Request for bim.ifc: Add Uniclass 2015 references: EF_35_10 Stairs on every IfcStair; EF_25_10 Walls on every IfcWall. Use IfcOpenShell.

First a look at what the model holds.

```python
import ifcopenshell

model = ifcopenshell.open("bim.ifc")
print(model.schema)
print("classifications:", [c.Name for c in model.by_type("IfcClassification")])
for ifc_class in ("IfcDoor", "IfcRoof", "IfcStair", "IfcWall", "IfcWindow"):
    print(ifc_class, len(model.by_type(ifc_class)))
```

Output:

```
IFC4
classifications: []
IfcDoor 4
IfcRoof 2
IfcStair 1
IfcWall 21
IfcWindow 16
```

```python
import ifcopenshell
import ifcopenshell.api.classification

model = ifcopenshell.open("bim.ifc")

system = ifcopenshell.api.classification.add_classification(model, classification="Uniclass 2015")

codes = {
    "IfcStair": ("EF_35_10", "Stairs"),
    "IfcWall": ("EF_25_10", "Walls"),
}
for ifc_class, (code, name) in codes.items():
    products = model.by_type(ifc_class)
    ifcopenshell.api.classification.add_reference(
        model, products=products, classification=system, identification=code, name=name
    )
    print(code, len(products))

model.write("bim_v2.ifc")
```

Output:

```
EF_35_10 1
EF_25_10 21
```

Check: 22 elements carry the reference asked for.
